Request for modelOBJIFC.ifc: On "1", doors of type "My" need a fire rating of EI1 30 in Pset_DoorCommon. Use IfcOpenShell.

First a look at what the model holds.

```python
import ifcopenshell
import ifcopenshell.util.element

model = ifcopenshell.open("modelOBJIFC.ifc")
print(model.schema)
storey = next(s for s in model.by_type("IfcBuildingStorey") if s.Name == "1")
doors = [e for e in ifcopenshell.util.element.get_decomposition(storey) if e.is_a("IfcDoor")]
seen = {}
for e in doors:
    element_type = ifcopenshell.util.element.get_type(e)
    key = (element_type.Name if element_type != e and element_type else None, ifcopenshell.util.element.get_pset(e, "Pset_DoorCommon", "FireRating"))
    seen[key] = seen.get(key, 0) + 1
for (name, value), count in sorted(seen.items(), key=str):
    print(count, "x", name, "|", value)
```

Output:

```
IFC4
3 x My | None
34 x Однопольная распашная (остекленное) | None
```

```python
import ifcopenshell
import ifcopenshell.api.pset
import ifcopenshell.util.element

model = ifcopenshell.open("modelOBJIFC.ifc")

storey = next(s for s in model.by_type("IfcBuildingStorey") if s.Name == "1")
doors = [e for e in ifcopenshell.util.element.get_decomposition(storey) if e.is_a("IfcDoor")]

count = 0
for e in doors:
    element_type = ifcopenshell.util.element.get_type(e)
    if element_type in (None, e) or element_type.Name != "My":
        continue
    # add_pset returns the element's existing set when there is one.
    pset = ifcopenshell.api.pset.add_pset(model, product=e, name="Pset_DoorCommon")
    ifcopenshell.api.pset.edit_pset(model, pset=pset, properties={"FireRating": "EI1 30"})
    count += 1

print(count, "doors updated")

model.write("modelOBJIFC-out.ifc")
```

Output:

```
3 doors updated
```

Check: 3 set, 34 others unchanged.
